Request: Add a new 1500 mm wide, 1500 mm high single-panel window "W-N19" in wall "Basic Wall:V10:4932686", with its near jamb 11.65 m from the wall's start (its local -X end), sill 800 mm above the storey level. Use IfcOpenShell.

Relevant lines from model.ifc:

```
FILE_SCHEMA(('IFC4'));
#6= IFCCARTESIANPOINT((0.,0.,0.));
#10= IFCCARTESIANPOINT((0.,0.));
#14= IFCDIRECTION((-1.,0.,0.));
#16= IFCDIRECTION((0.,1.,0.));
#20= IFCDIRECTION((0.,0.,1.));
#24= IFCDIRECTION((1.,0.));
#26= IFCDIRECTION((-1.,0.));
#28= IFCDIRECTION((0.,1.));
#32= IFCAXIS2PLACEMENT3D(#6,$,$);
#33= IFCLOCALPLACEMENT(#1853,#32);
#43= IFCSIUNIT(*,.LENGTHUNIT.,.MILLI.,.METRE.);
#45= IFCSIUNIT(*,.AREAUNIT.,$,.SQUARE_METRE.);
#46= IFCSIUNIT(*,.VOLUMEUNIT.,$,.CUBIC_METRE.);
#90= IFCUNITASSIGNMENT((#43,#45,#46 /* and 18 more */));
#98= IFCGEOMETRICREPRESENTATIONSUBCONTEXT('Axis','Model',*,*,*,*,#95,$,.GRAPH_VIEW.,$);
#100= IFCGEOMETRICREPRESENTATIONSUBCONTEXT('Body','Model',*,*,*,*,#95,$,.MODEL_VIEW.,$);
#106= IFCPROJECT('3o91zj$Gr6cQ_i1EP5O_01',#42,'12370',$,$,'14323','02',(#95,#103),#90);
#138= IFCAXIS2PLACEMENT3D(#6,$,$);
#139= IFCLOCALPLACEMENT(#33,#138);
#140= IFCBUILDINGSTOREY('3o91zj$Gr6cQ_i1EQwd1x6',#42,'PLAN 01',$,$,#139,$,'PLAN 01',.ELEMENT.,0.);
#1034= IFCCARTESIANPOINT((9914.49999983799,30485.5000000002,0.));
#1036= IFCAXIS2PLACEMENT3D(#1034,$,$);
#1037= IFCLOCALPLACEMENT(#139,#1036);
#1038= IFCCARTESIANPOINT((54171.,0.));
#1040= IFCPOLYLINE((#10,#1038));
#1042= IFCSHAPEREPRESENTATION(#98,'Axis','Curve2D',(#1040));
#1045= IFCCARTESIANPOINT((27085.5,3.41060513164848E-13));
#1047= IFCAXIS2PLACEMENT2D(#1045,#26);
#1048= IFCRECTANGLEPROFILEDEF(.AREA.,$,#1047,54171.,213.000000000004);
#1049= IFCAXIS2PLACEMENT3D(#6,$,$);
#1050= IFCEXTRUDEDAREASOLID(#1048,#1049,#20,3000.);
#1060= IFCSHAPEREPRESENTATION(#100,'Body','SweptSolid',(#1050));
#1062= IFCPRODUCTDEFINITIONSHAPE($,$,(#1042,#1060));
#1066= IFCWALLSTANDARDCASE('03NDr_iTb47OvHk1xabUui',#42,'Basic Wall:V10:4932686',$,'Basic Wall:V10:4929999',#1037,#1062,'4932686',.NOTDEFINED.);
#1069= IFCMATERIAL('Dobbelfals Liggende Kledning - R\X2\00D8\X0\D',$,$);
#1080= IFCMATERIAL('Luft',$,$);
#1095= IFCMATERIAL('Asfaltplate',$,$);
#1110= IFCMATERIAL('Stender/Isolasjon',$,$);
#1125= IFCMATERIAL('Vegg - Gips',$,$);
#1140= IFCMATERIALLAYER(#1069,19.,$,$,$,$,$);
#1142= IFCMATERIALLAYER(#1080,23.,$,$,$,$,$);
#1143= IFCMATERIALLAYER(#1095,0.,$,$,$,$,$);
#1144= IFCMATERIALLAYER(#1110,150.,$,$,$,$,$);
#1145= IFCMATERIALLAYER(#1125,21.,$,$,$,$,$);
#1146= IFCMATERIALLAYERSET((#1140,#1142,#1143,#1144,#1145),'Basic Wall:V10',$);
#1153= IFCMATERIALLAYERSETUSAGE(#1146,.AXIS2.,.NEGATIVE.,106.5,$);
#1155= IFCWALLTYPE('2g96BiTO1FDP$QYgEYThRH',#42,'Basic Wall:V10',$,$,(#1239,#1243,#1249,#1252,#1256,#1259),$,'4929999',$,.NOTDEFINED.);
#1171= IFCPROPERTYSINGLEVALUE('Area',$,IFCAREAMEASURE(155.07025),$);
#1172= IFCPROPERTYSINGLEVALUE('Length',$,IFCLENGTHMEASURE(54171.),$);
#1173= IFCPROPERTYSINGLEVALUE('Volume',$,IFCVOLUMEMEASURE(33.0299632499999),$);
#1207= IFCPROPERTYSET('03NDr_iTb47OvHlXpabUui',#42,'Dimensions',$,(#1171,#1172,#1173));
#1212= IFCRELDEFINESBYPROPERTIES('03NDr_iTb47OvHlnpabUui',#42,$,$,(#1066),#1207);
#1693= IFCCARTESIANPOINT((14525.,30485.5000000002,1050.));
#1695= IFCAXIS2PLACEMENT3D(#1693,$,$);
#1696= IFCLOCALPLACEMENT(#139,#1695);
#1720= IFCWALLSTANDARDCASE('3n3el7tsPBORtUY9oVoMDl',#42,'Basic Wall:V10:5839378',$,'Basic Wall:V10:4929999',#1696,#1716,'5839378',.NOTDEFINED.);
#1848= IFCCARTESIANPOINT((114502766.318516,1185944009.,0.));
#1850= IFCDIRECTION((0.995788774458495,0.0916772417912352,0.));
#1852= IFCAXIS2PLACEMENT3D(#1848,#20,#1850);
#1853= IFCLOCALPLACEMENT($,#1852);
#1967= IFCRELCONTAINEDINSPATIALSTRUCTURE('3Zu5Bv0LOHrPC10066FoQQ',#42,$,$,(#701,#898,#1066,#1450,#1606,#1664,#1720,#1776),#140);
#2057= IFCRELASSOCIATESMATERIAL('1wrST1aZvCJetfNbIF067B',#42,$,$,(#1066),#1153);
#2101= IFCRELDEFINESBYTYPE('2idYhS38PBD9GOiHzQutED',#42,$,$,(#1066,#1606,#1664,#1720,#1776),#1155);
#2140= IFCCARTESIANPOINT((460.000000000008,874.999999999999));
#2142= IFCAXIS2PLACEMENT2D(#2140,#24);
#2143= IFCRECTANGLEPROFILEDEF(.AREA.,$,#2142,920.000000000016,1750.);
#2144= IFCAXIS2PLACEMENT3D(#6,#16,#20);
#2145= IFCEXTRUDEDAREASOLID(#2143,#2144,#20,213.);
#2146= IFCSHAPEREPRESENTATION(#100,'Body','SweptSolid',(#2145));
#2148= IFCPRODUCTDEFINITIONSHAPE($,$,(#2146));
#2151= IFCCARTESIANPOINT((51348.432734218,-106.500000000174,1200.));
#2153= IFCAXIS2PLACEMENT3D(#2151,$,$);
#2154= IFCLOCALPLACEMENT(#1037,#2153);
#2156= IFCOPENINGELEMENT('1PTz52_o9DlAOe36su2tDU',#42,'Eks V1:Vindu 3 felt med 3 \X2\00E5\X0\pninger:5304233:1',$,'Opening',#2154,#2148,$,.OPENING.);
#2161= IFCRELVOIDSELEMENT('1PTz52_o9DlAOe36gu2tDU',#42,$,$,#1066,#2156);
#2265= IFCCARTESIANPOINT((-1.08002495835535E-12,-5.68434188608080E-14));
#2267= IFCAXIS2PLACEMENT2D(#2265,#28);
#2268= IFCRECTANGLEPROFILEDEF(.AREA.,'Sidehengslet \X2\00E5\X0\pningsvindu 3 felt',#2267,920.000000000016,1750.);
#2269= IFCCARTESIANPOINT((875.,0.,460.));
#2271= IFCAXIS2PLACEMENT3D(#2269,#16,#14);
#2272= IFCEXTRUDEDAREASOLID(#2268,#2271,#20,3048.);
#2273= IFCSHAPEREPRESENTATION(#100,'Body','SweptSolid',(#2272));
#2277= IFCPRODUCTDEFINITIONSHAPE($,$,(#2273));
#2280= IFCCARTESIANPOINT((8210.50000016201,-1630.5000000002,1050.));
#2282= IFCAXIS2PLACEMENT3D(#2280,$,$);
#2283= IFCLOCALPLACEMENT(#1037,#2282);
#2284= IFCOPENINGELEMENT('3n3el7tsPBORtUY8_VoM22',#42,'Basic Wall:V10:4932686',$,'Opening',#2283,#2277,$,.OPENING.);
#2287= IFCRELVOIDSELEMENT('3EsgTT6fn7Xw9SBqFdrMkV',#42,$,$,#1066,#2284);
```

```python
import numpy as np
import ifcopenshell
import ifcopenshell.api.feature
import ifcopenshell.api.geometry
import ifcopenshell.api.pset
import ifcopenshell.api.root
import ifcopenshell.api.spatial
import ifcopenshell.geom
import ifcopenshell.util.element
import ifcopenshell.util.placement
import ifcopenshell.util.representation
import ifcopenshell.util.shape
import ifcopenshell.util.unit

model = ifcopenshell.open("model.ifc")
unit_scale = ifcopenshell.util.unit.calculate_unit_scale(model)
area_scale = ifcopenshell.util.unit.calculate_unit_scale(model, "AREAUNIT")
volume_scale = ifcopenshell.util.unit.calculate_unit_scale(model, "VOLUMEUNIT")
settings = ifcopenshell.geom.settings()


def volume(element):
    """Net volume in cubic metres, openings subtracted."""
    shape = ifcopenshell.geom.create_shape(settings, element)
    return ifcopenshell.util.shape.get_volume(shape.geometry)


wall = model.by_id(1066)
storey = ifcopenshell.util.element.get_container(wall, ifc_class="IfcBuildingStorey")
context = ifcopenshell.util.representation.get_context(model, "Model", "Body", "MODEL_VIEW")
before = volume(wall)

width, height, from_end, sill = 1.5, 1.5, 11.65, 0.8  # metres

# The wall runs along its own X axis, and the end named is its -X end.
wall_shape = ifcopenshell.geom.create_shape(settings, wall)
x, y, z = ifcopenshell.util.shape.get_vertices(wall_shape.geometry).T
start = x.min() + from_end
face, thickness = float(y.min()), float(y.max() - y.min())
wall_matrix = ifcopenshell.util.placement.get_local_placement(wall.ObjectPlacement)
level = ifcopenshell.util.placement.get_local_placement(storey.ObjectPlacement)[2, 3]


def in_wall(x, y):
    """Placement at x, y metres in the wall's axes, at sill height."""
    matrix = wall_matrix.copy()
    matrix[:, 3] = wall_matrix @ np.array([x / unit_scale, y / unit_scale, 0.0, 1.0])
    matrix[2, 3] = level + sill / unit_scale
    return matrix


# Opening: a box that overshoots both wall faces by 50 mm.
opening = ifcopenshell.api.root.create_entity(model, ifc_class="IfcOpeningElement", predefined_type="OPENING")
box = ifcopenshell.api.geometry.add_wall_representation(
    model, context=context, length=width, height=height, thickness=thickness + 0.1
)
ifcopenshell.api.geometry.assign_representation(model, product=opening, representation=box)
ifcopenshell.api.geometry.edit_object_placement(model, product=opening, matrix=in_wall(start, face - 0.05), is_si=False)
ifcopenshell.api.feature.add_feature(model, feature=opening, element=wall)

window = ifcopenshell.api.root.create_entity(model, ifc_class="IfcWindow", name="W-N19", predefined_type="WINDOW")
window.OverallWidth, window.OverallHeight = width / unit_scale, height / unit_scale
window.PartitioningType = "SINGLE_PANEL"
body = ifcopenshell.api.geometry.add_window_representation(
    model,
    context=context,
    overall_width=window.OverallWidth,
    overall_height=window.OverallHeight,
    partition_type="SINGLE_PANEL",
)
ifcopenshell.api.geometry.assign_representation(model, product=window, representation=body)
ifcopenshell.api.spatial.assign_container(model, products=[window], relating_structure=storey)
ifcopenshell.api.feature.add_filling(model, opening=opening, element=window)

# Centre the window in the wall's thickness.
ifcopenshell.api.geometry.edit_object_placement(model, product=window, matrix=in_wall(start, face), is_si=False)
window_shape = ifcopenshell.geom.create_shape(settings, window)
depth = ifcopenshell.util.shape.get_vertices(window_shape.geometry)[:, 1]
offset = face + thickness / 2 - (depth.min() + depth.max()) / 2
ifcopenshell.api.geometry.edit_object_placement(model, product=window, matrix=in_wall(start, offset), is_si=False)

after = volume(wall)

# Update the wall's stored quantities.
pset = model.by_id(ifcopenshell.util.element.get_pset(wall, "Dimensions", should_inherit=False)["id"])
ifcopenshell.api.pset.edit_pset(model, pset=pset, properties={
    "Area": model.create_entity("IfcAreaMeasure", after / thickness / area_scale),
    "Volume": model.create_entity("IfcVolumeMeasure", after / volume_scale),
})

print(f"wall volume {before:.3f} -> {after:.3f} m3")

model.write("model_v2.ifc")
```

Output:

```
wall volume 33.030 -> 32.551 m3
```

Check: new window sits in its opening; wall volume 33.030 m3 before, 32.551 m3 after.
